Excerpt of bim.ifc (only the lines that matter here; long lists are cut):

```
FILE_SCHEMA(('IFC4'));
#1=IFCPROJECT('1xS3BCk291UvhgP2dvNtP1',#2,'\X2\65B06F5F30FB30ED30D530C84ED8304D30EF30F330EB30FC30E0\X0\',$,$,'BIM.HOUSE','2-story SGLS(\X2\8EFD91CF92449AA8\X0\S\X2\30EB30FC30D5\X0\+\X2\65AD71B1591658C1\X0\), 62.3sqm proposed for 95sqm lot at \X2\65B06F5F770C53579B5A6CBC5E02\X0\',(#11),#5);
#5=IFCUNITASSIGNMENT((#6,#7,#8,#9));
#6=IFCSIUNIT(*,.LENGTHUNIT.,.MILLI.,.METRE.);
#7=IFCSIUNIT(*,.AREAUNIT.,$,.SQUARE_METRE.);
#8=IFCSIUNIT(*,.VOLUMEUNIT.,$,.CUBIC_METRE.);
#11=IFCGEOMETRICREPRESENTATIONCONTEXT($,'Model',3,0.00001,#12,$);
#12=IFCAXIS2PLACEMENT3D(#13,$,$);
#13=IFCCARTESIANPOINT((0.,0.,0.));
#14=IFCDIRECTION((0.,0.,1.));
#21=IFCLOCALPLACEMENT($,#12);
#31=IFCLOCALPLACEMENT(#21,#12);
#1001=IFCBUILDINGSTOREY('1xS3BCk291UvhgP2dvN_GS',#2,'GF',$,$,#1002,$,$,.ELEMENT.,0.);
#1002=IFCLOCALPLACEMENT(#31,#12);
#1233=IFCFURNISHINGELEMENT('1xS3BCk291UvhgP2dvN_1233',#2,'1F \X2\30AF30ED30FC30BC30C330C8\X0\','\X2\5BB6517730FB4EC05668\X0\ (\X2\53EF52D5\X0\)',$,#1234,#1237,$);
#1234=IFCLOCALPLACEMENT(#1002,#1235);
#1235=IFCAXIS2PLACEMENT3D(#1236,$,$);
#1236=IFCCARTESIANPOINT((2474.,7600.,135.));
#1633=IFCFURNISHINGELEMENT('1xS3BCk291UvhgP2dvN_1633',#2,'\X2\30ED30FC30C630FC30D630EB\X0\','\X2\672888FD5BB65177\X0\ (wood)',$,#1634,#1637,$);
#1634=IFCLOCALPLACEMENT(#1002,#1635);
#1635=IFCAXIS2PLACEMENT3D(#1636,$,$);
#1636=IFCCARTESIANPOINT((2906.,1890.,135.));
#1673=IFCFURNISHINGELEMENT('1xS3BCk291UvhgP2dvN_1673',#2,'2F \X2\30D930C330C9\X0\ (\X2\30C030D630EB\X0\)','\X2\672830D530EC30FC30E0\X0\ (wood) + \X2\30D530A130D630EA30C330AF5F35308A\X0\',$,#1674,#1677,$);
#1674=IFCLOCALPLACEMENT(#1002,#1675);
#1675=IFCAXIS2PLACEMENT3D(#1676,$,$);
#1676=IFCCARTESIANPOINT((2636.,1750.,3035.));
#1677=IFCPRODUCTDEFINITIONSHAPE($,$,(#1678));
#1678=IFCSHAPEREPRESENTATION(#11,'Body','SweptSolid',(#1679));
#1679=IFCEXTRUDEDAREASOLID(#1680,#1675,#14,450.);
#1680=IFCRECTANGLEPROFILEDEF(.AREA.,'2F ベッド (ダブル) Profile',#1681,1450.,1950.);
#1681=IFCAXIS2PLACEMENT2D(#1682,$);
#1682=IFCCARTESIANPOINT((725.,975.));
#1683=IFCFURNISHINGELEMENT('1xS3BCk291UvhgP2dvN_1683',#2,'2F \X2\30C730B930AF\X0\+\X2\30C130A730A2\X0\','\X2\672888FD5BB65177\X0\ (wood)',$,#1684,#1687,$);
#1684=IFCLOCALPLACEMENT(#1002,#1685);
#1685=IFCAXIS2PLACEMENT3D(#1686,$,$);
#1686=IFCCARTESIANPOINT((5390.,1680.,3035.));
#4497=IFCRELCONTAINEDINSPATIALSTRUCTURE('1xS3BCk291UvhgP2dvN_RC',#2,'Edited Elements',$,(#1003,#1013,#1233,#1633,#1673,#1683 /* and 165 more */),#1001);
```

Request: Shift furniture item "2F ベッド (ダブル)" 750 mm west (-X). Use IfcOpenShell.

```python
import ifcopenshell
import ifcopenshell.api.geometry
import ifcopenshell.util.placement

model = ifcopenshell.open("bim.ifc")

item = model.by_guid("1xS3BCk291UvhgP2dvN_1673")
matrix = ifcopenshell.util.placement.get_local_placement(item.ObjectPlacement)
matrix[0, 3] -= 750.0
ifcopenshell.api.geometry.edit_object_placement(model, product=item, matrix=matrix, is_si=False)

print(ifcopenshell.util.placement.get_local_placement(item.ObjectPlacement).round(3) + 0.0)

model.write("bim-out.ifc")
```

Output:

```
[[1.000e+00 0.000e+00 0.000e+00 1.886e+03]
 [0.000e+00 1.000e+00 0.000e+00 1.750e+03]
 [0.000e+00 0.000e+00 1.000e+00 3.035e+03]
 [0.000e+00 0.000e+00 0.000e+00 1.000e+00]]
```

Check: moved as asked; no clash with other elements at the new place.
